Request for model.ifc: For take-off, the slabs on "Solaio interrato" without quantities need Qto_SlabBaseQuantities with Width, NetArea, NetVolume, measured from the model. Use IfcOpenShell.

First a look at what the model holds.

```python
import ifcopenshell
import ifcopenshell.util.element
import ifcopenshell.util.unit

model = ifcopenshell.open("model.ifc")
print(model.schema)
for unit_type in ("LENGTHUNIT", "AREAUNIT", "VOLUMEUNIT"):
    print(unit_type, ifcopenshell.util.unit.calculate_unit_scale(model, unit_type))
storey = next(s for s in model.by_type("IfcBuildingStorey") if s.Name == "Solaio interrato")
slabs = [e for e in ifcopenshell.util.element.get_decomposition(storey) if e.is_a("IfcSlab")]
for e in sorted(slabs, key=lambda e: e.id()):
    print(e.id(), e.is_a(), e.Name, list(ifcopenshell.util.element.get_psets(e, qtos_only=True)), sep=" | ")
```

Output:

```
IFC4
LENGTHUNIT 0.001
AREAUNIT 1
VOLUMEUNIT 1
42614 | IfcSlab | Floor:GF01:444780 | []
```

```python
import ifcopenshell
import ifcopenshell.api.pset
import ifcopenshell.geom
import ifcopenshell.util.element
import ifcopenshell.util.shape
import ifcopenshell.util.unit

model = ifcopenshell.open("model.ifc")
unit_scale = ifcopenshell.util.unit.calculate_unit_scale(model)
area_scale = ifcopenshell.util.unit.calculate_unit_scale(model, "AREAUNIT")
volume_scale = ifcopenshell.util.unit.calculate_unit_scale(model, "VOLUMEUNIT")
settings = ifcopenshell.geom.settings()

storey = next(s for s in model.by_type("IfcBuildingStorey") if s.Name == "Solaio interrato")
slabs = [e for e in ifcopenshell.util.element.get_decomposition(storey) if e.is_a("IfcSlab")]

for e in sorted(slabs, key=lambda e: e.id()):
    if ifcopenshell.util.element.get_psets(e, qtos_only=True, should_inherit=False):
        continue
    # Geometry comes back in metres, in the element's own axes.
    shape = ifcopenshell.geom.create_shape(settings, e)
    values = {
        "Width": ifcopenshell.util.shape.get_z(shape.geometry) / unit_scale,
        "NetArea": ifcopenshell.util.shape.get_footprint_area(shape.geometry) / area_scale,
        "NetVolume": ifcopenshell.util.shape.get_volume(shape.geometry) / volume_scale,
    }
    qto = ifcopenshell.api.pset.add_qto(model, product=e, name="Qto_SlabBaseQuantities")
    ifcopenshell.api.pset.edit_qto(model, qto=qto, properties=values)
    print(e.id(), {k: round(v, 3) for k, v in values.items()})

model.write("model_rev.ifc")
```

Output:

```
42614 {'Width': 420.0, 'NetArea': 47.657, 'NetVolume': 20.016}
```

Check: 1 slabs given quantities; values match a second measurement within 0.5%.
